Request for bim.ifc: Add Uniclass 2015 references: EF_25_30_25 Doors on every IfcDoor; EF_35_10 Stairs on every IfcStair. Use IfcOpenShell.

First a look at what the model holds.

```python
import ifcopenshell

model = ifcopenshell.open("bim.ifc")
print(model.schema)
print("classifications:", [c.Name for c in model.by_type("IfcClassification")])
for ifc_class in ("IfcDoor", "IfcRoof", "IfcStair", "IfcWall", "IfcWindow"):
    print(ifc_class, len(model.by_type(ifc_class)))
```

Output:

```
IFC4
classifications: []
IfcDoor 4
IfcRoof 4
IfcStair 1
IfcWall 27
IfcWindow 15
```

```python
import ifcopenshell
import ifcopenshell.api.classification

model = ifcopenshell.open("bim.ifc")

system = ifcopenshell.api.classification.add_classification(model, classification="Uniclass 2015")

codes = {
    "IfcDoor": ("EF_25_30_25", "Doors"),
    "IfcStair": ("EF_35_10", "Stairs"),
}
for ifc_class, (code, name) in codes.items():
    products = model.by_type(ifc_class)
    ifcopenshell.api.classification.add_reference(
        model, products=products, classification=system, identification=code, name=name
    )
    print(code, len(products))

model.write("bim-out.ifc")
```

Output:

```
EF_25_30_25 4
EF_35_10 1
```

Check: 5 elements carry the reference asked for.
